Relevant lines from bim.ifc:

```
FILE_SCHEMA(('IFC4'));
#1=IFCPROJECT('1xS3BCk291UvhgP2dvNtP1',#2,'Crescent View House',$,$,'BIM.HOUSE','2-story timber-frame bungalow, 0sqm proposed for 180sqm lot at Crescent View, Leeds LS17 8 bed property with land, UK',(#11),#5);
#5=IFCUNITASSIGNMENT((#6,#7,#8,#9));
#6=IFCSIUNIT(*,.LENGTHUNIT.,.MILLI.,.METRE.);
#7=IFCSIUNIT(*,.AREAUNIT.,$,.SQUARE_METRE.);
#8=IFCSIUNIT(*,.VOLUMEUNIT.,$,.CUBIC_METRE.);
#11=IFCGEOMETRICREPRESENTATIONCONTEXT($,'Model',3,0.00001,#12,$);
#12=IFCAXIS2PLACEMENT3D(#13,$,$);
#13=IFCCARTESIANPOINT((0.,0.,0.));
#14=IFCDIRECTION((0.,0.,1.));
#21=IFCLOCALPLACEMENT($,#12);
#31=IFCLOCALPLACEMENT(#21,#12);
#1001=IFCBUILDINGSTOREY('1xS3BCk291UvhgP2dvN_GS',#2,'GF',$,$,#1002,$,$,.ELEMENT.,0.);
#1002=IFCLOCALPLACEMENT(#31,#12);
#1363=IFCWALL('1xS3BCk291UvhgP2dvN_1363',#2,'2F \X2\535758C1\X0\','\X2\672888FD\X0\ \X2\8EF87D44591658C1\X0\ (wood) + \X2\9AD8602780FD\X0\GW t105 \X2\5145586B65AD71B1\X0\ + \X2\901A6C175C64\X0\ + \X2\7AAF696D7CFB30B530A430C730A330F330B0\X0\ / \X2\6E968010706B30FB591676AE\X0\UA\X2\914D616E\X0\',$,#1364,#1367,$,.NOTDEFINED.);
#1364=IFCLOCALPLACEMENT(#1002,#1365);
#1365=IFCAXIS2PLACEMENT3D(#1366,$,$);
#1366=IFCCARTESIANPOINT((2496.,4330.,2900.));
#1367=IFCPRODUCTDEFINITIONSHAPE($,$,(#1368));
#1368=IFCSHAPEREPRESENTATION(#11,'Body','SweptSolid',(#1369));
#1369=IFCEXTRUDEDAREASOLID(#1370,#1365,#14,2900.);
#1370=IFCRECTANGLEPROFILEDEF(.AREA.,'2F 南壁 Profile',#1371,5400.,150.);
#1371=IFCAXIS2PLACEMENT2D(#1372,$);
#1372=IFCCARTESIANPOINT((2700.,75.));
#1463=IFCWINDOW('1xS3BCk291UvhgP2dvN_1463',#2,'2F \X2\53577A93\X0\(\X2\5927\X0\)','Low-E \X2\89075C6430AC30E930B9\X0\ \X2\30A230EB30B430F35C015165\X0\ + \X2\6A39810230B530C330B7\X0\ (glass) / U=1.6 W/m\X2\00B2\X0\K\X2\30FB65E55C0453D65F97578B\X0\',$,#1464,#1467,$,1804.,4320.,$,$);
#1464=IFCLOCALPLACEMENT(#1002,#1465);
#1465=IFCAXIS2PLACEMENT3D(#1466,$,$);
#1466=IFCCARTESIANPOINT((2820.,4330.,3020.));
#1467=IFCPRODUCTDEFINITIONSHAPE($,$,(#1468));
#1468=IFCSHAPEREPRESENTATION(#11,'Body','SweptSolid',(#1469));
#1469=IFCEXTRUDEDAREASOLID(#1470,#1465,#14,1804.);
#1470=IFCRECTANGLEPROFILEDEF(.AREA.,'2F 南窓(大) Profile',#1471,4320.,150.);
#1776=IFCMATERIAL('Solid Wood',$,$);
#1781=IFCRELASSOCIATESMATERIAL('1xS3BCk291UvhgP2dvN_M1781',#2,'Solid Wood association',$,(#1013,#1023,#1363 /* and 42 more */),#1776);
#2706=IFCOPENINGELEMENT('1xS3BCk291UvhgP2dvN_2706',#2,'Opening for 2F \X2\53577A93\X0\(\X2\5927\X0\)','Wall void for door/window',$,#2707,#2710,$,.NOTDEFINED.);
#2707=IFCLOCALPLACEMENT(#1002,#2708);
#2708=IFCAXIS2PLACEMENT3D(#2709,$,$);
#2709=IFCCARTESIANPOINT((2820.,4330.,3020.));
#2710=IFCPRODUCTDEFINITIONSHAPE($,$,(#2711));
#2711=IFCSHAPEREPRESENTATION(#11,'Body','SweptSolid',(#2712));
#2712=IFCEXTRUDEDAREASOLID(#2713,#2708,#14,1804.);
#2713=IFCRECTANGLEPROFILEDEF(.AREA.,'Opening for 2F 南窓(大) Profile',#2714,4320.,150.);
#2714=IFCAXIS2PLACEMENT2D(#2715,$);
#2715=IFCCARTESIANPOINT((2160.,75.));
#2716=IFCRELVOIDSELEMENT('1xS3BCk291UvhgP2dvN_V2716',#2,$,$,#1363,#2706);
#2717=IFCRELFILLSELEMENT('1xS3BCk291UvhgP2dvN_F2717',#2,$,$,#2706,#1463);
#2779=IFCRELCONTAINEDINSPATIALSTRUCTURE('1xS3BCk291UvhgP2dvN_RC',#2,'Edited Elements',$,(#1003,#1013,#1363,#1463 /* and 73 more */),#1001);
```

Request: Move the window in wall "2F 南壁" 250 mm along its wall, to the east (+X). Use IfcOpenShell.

```python
import ifcopenshell
import ifcopenshell.api.geometry
import ifcopenshell.util.placement

model = ifcopenshell.open("bim.ifc")

window = model.by_id(1463)
opening = window.FillsVoids[0].RelatingOpeningElement
wall = opening.VoidsElements[0].RelatingBuildingElement

wall_matrix = ifcopenshell.util.placement.get_local_placement(wall.ObjectPlacement)
shift = wall_matrix[:3, 0] * 250.0
before = ifcopenshell.util.placement.get_local_placement(window.ObjectPlacement)[:3, 3].copy()

# The window is not placed relative to its opening, so move both.
for product in (opening, window):
    matrix = ifcopenshell.util.placement.get_local_placement(product.ObjectPlacement)
    matrix[:3, 3] += shift
    ifcopenshell.api.geometry.edit_object_placement(model, product=product, matrix=matrix, is_si=False)

after = ifcopenshell.util.placement.get_local_placement(window.ObjectPlacement)[:3, 3]
print("window moved by", (after - before).round(3) + 0.0)

model.write("bim_updated.ifc")
```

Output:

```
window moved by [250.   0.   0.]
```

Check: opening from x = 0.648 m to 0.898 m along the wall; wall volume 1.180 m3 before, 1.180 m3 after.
